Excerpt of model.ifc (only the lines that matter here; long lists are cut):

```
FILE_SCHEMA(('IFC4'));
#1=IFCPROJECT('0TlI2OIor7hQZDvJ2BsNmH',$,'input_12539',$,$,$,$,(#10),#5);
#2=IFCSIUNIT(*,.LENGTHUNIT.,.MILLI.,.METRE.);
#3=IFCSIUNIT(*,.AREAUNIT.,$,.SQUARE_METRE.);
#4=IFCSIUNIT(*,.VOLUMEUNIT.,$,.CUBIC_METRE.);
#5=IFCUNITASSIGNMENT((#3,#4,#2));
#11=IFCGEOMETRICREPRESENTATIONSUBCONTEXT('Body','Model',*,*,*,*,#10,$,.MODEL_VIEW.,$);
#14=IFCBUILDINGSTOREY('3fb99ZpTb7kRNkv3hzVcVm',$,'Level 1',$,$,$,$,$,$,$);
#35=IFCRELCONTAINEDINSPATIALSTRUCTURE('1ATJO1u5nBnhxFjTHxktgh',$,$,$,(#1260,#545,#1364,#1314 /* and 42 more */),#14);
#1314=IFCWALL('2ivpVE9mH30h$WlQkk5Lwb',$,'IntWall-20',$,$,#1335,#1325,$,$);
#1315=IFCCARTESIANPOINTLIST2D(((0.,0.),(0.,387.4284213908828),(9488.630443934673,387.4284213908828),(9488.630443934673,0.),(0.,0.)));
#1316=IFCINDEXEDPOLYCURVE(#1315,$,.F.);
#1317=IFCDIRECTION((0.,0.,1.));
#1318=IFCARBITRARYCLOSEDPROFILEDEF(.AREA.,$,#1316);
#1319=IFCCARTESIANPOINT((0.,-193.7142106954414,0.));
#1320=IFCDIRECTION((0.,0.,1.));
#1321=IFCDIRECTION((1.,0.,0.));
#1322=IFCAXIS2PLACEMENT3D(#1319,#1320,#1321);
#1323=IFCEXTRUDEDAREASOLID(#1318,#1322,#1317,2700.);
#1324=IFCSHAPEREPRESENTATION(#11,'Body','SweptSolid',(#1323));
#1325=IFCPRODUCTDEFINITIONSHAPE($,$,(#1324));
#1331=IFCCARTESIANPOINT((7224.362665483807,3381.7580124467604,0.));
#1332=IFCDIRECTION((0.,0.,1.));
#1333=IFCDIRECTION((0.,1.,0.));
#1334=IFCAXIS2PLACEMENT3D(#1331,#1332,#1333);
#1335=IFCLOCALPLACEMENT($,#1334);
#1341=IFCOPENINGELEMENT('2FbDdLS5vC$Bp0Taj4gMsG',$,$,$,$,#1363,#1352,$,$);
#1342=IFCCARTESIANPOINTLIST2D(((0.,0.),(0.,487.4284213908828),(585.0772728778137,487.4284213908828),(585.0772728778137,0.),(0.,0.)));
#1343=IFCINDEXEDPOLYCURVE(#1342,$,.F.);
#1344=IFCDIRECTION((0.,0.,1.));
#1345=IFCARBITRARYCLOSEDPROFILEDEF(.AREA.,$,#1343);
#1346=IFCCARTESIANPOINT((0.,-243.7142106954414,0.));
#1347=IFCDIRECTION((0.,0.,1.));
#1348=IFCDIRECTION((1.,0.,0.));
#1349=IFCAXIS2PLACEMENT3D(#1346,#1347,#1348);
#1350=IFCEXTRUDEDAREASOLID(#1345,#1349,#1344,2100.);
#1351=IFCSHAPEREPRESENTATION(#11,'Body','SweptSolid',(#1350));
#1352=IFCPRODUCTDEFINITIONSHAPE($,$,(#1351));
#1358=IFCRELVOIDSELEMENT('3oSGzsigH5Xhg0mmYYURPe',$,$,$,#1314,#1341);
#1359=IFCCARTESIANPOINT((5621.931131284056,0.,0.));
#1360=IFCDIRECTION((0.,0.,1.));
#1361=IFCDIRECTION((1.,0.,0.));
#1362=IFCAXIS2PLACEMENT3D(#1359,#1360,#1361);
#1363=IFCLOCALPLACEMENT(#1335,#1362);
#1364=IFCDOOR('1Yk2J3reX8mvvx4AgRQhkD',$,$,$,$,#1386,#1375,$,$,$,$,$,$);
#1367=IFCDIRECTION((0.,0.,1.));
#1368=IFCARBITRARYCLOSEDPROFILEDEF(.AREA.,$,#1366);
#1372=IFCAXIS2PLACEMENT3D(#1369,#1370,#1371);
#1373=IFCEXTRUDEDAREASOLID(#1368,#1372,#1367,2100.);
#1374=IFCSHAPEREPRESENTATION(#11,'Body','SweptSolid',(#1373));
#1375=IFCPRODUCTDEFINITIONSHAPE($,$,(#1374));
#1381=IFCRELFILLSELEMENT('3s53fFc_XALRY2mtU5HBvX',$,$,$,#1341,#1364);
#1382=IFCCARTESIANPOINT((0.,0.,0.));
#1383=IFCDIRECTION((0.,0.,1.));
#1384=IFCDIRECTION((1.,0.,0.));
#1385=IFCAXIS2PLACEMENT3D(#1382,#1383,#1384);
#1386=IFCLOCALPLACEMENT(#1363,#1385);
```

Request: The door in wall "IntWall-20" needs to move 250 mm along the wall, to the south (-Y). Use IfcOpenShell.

```python
import ifcopenshell
import ifcopenshell.api.geometry
import ifcopenshell.util.placement
import ifcopenshell.util.unit

model = ifcopenshell.open("model.ifc")
unit_scale = ifcopenshell.util.unit.calculate_unit_scale(model)

door = model.by_guid("1Yk2J3reX8mvvx4AgRQhkD")
opening = door.FillsVoids[0].RelatingOpeningElement
wall = opening.VoidsElements[0].RelatingBuildingElement

wall_matrix = ifcopenshell.util.placement.get_local_placement(wall.ObjectPlacement)
shift = wall_matrix[:3, 0] * -0.25 / unit_scale
before = ifcopenshell.util.placement.get_local_placement(door.ObjectPlacement)[:3, 3].copy()

# The door is placed relative to its opening, so it follows when the opening moves.
matrix = ifcopenshell.util.placement.get_local_placement(opening.ObjectPlacement)
matrix[:3, 3] += shift
ifcopenshell.api.geometry.edit_object_placement(
    model, product=opening, matrix=matrix, is_si=False, should_transform_children=True
)

after = ifcopenshell.util.placement.get_local_placement(door.ObjectPlacement)[:3, 3]
print("door moved by", (after - before).round(3) + 0.0)

model.write("model_edited.ifc")
```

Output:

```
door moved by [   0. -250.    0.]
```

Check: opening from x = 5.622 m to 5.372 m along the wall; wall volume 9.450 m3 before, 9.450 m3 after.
